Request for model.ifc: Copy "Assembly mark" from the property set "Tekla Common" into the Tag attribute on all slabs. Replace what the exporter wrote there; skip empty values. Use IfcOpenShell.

First a look at what the model holds.

```python
import ifcopenshell
import ifcopenshell.util.element

model = ifcopenshell.open("model.ifc")
print(model.schema)
slabs = model.by_type("IfcSlab")
print(len(slabs), "slabs")
for e in slabs[:8]:
    source = ifcopenshell.util.element.get_pset(e, "Tekla Common", "Assembly mark")
    target = e.Tag
    print(e.id(), repr(source), repr(target), sep=" | ")
```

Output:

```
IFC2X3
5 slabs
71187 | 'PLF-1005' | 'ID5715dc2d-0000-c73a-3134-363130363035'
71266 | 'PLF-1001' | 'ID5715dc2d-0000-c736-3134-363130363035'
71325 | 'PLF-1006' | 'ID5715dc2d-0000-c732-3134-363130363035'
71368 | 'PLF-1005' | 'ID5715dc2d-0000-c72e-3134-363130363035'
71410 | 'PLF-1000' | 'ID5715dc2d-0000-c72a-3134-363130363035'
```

```python
import ifcopenshell
import ifcopenshell.util.element

model = ifcopenshell.open("model.ifc")

count = 0
for e in model.by_type("IfcSlab"):
    value = ifcopenshell.util.element.get_pset(e, "Tekla Common", "Assembly mark")
    current = e.Tag
    if not value or not value.strip() or current == value:
        continue
    e.Tag = value
    count += 1

print(count, "slabs updated")

model.write("model_edited.ifc")
```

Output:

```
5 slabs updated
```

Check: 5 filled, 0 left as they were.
